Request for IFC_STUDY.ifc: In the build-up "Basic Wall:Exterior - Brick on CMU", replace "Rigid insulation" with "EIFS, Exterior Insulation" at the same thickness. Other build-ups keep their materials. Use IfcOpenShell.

First a look at what the model holds.

```python
import ifcopenshell
import ifcopenshell.util.element

model = ifcopenshell.open("IFC_STUDY.ifc")
print(model.schema)
for layer_set in model.by_type("IfcMaterialLayerSet"):
    if layer_set.LayerSetName == "Basic Wall:Exterior - Brick on CMU":
        for layer in layer_set.MaterialLayers:
            print(layer.id(), layer.Material and layer.Material.Name, layer.LayerThickness, sep=" | ")
        print(len(ifcopenshell.util.element.get_elements_by_material(model, layer_set)), "elements and types use it")
print(sorted(m.Name for m in model.by_type("IfcMaterial") if m.Name)[:60])
```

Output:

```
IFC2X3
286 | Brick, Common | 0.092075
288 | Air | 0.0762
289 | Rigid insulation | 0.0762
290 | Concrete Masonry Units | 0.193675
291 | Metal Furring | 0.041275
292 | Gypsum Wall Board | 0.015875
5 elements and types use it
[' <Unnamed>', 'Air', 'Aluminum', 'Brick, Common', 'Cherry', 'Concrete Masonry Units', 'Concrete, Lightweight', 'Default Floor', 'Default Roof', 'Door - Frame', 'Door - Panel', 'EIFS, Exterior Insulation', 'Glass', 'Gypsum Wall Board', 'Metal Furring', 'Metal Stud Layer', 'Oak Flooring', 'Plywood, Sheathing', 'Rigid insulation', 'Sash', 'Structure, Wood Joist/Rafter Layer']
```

```python
import ifcopenshell
import ifcopenshell.api.material

model = ifcopenshell.open("IFC_STUDY.ifc")

layer_set = next(s for s in model.by_type("IfcMaterialLayerSet") if s.LayerSetName == "Basic Wall:Exterior - Brick on CMU")
layer = next(l for l in layer_set.MaterialLayers if l.Material and l.Material.Name == "Rigid insulation")
material = next(m for m in model.by_type("IfcMaterial") if m.Name == "EIFS, Exterior Insulation")

# Point this one layer at the other material; renaming the old one would change it everywhere.
ifcopenshell.api.material.edit_layer(model, layer=layer, attributes={}, material=material)

print([l.Material.Name if l.Material else None for l in layer_set.MaterialLayers])

model.write("IFC_STUDY_rev.ifc")
```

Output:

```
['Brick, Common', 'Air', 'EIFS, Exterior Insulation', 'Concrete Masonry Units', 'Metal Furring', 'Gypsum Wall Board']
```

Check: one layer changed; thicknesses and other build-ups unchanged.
